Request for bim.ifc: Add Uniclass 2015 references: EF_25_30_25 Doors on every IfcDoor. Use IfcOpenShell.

First a look at what the model holds.

```python
import ifcopenshell

model = ifcopenshell.open("bim.ifc")
print(model.schema)
print("classifications:", [c.Name for c in model.by_type("IfcClassification")])
for ifc_class in ("IfcDoor", "IfcRoof", "IfcStair", "IfcWall", "IfcWindow"):
    print(ifc_class, len(model.by_type(ifc_class)))
```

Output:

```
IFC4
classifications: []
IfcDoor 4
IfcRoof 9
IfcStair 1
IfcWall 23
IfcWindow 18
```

```python
import ifcopenshell
import ifcopenshell.api.classification

model = ifcopenshell.open("bim.ifc")

system = ifcopenshell.api.classification.add_classification(model, classification="Uniclass 2015")

codes = {
    "IfcDoor": ("EF_25_30_25", "Doors"),
}
for ifc_class, (code, name) in codes.items():
    products = model.by_type(ifc_class)
    ifcopenshell.api.classification.add_reference(
        model, products=products, classification=system, identification=code, name=name
    )
    print(code, len(products))

model.write("bim_v2.ifc")
```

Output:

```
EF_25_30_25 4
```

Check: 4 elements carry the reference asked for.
